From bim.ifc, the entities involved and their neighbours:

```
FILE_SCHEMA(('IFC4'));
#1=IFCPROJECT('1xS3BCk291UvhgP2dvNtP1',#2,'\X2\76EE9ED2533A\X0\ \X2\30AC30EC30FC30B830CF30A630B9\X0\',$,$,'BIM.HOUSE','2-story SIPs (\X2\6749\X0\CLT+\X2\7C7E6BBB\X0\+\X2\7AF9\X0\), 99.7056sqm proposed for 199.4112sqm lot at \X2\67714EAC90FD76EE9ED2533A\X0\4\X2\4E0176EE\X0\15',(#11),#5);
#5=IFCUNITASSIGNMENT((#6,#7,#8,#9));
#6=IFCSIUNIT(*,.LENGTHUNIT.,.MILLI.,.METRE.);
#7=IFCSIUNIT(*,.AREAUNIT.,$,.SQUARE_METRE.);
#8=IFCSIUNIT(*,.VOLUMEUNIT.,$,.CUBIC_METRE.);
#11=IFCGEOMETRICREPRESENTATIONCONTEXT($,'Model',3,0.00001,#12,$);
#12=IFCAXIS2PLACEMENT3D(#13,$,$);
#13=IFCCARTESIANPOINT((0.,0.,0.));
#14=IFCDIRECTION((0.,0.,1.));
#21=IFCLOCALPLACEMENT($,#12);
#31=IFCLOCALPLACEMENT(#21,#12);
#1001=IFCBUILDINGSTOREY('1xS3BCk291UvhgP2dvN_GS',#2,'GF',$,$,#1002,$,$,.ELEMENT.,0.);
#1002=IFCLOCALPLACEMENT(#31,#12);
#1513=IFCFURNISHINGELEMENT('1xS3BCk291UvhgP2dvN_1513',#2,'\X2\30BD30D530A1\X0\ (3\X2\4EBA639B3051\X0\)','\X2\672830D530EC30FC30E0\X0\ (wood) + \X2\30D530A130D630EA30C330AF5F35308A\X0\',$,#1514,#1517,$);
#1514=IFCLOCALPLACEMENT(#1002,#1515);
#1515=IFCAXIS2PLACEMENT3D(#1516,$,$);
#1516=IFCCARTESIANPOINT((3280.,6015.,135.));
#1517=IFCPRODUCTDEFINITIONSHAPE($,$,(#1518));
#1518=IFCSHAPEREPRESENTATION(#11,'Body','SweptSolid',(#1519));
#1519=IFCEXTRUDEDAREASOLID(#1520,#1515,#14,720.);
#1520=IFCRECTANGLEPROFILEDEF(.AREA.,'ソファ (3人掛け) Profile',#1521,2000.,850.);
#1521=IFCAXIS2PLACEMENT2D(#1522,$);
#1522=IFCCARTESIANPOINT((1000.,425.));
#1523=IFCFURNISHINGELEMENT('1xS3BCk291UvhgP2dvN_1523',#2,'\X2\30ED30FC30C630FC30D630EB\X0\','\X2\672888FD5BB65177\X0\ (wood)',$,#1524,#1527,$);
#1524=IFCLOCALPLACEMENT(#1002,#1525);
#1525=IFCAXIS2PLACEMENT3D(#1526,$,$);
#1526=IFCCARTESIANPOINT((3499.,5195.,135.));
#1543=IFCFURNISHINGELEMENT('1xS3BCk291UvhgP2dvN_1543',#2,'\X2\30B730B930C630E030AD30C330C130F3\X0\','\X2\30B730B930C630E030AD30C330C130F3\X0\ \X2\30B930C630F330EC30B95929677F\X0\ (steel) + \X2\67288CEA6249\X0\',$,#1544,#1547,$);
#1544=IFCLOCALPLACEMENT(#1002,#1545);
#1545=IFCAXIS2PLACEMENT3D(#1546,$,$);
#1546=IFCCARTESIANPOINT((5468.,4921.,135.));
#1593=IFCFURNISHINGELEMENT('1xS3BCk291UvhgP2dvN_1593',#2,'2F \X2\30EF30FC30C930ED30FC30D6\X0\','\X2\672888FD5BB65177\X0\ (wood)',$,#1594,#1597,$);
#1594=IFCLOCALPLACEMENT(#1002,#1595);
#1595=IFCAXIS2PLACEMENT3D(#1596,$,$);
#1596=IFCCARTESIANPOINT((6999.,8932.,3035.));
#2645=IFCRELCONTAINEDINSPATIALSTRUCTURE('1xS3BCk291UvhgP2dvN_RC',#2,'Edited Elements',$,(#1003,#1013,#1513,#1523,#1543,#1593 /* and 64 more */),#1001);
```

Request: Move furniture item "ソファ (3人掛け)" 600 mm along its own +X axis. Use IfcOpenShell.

```python
import ifcopenshell
import ifcopenshell.api.geometry
import ifcopenshell.util.placement
import ifcopenshell.util.unit

model = ifcopenshell.open("bim.ifc")
unit_scale = ifcopenshell.util.unit.calculate_unit_scale(model)

item = model.by_guid("1xS3BCk291UvhgP2dvN_1513")
matrix = ifcopenshell.util.placement.get_local_placement(item.ObjectPlacement)
matrix[:3, 3] += matrix[:3, 0] * 0.6 / unit_scale
ifcopenshell.api.geometry.edit_object_placement(model, product=item, matrix=matrix, is_si=False)

print(ifcopenshell.util.placement.get_local_placement(item.ObjectPlacement).round(3) + 0.0)

model.write("bim_rev.ifc")
```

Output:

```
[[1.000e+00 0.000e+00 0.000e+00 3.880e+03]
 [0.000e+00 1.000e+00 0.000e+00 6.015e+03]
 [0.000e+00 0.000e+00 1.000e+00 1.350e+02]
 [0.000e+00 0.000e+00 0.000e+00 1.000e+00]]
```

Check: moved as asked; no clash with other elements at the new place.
